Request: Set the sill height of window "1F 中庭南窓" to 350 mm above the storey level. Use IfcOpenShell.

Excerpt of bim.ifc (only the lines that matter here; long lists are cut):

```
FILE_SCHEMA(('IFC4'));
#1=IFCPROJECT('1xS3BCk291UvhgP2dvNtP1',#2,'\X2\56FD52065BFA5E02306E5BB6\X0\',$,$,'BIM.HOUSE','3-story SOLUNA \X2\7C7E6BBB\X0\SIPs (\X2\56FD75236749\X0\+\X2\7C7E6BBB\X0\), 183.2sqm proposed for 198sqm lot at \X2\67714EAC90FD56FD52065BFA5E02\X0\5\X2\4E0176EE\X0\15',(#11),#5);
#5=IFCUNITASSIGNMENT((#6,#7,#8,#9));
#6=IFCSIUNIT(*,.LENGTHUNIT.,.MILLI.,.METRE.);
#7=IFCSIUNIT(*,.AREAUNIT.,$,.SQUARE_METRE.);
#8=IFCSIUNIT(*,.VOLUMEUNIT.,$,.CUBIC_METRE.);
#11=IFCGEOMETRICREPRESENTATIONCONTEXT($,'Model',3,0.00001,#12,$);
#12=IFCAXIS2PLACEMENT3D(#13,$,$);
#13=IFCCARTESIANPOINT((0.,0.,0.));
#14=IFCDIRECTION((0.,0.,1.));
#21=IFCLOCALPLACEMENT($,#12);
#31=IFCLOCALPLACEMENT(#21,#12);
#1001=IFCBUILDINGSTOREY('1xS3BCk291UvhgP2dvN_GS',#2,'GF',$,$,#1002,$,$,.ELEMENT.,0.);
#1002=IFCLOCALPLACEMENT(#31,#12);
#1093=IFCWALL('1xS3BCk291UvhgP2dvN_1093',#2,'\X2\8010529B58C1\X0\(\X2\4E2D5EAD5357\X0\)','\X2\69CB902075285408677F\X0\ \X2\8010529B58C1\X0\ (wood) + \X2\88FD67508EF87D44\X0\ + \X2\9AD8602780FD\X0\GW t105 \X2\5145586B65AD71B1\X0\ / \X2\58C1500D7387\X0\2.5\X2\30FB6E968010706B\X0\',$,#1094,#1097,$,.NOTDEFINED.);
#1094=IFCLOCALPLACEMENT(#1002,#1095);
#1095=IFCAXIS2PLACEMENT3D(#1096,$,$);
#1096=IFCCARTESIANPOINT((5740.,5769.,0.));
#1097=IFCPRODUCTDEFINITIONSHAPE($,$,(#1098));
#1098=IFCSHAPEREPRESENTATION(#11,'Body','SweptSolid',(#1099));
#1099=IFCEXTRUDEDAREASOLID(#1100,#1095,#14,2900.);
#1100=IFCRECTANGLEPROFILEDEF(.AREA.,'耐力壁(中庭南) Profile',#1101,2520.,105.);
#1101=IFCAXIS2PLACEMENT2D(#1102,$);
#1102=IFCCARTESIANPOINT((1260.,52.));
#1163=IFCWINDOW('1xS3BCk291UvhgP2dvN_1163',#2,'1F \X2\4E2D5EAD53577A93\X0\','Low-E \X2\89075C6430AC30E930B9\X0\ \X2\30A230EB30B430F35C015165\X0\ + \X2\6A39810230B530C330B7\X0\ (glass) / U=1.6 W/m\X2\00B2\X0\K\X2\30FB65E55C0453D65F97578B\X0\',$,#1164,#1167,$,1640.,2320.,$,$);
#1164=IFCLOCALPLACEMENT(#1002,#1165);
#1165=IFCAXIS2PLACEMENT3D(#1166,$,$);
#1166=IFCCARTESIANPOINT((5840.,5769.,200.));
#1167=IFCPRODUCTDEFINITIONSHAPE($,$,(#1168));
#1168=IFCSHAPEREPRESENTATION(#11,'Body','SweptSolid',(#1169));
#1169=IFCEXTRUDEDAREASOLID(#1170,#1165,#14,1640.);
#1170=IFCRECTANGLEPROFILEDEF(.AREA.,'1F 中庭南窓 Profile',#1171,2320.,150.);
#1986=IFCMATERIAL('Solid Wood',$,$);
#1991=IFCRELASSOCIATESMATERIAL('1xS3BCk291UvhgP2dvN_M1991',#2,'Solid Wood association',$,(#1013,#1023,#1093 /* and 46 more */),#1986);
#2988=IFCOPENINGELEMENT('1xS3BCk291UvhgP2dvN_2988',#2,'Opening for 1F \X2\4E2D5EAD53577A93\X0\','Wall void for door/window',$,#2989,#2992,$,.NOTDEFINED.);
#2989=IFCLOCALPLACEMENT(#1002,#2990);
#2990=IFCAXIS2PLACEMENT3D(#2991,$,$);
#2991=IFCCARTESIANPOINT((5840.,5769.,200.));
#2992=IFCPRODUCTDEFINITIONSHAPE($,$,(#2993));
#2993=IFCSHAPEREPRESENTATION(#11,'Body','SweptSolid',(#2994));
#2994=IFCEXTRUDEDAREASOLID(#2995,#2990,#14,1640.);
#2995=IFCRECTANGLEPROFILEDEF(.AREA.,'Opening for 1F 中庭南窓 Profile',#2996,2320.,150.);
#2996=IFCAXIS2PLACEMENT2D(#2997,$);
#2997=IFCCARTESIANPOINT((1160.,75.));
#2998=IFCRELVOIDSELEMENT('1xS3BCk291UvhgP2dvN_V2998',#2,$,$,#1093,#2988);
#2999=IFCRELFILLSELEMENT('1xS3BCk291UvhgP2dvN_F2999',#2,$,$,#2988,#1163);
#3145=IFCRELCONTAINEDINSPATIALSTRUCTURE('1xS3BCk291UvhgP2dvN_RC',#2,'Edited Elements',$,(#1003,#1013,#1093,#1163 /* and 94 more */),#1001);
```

```python
import numpy as np
import ifcopenshell
import ifcopenshell.api.geometry
import ifcopenshell.geom
import ifcopenshell.util.element
import ifcopenshell.util.placement
import ifcopenshell.util.shape
import ifcopenshell.util.unit

model = ifcopenshell.open("bim.ifc")
unit_scale = ifcopenshell.util.unit.calculate_unit_scale(model)

window = model.by_guid("1xS3BCk291UvhgP2dvN_1163")
opening = window.FillsVoids[0].RelatingOpeningElement
storey = ifcopenshell.util.element.get_container(window, ifc_class="IfcBuildingStorey")
level = ifcopenshell.util.placement.get_local_placement(storey.ObjectPlacement)[2, 3]

# The opening's origin need not be at the sill, so measure its lowest point.
shape = ifcopenshell.geom.create_shape(ifcopenshell.geom.settings(), opening)
bottom = ifcopenshell.util.shape.get_shape_bottom_elevation(shape, shape.geometry) / unit_scale
dz = level + 0.35 / unit_scale - bottom

shift = np.array([0.0, 0.0, dz])
# The window is not placed relative to its opening, so move both.
for product in (opening, window):
    matrix = ifcopenshell.util.placement.get_local_placement(product.ObjectPlacement)
    matrix[:3, 3] += shift
    ifcopenshell.api.geometry.edit_object_placement(model, product=product, matrix=matrix, is_si=False)

print(f"moved by {dz * unit_scale:+.3f} m")

model.write("bim_v2.ifc")
```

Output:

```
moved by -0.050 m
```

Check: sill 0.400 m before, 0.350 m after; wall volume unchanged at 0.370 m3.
